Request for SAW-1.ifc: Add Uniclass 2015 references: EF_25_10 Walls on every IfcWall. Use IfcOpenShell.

First a look at what the model holds.

```python
import ifcopenshell

model = ifcopenshell.open("SAW-1.ifc")
print(model.schema)
print("classifications:", [c.Name for c in model.by_type("IfcClassification")])
for ifc_class in ("IfcDoor", "IfcRoof", "IfcStair", "IfcWall", "IfcWindow"):
    print(ifc_class, len(model.by_type(ifc_class)))
```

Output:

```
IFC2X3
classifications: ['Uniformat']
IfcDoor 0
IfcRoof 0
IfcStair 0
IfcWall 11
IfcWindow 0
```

```python
import ifcopenshell
import ifcopenshell.api.classification

model = ifcopenshell.open("SAW-1.ifc")

# IFC2X3 requires Source and Edition and has no link from the project to the system.
system = model.create_entity("IfcClassification", Source="NBS", Edition="2015", Name="Uniclass 2015")

codes = {
    "IfcWall": ("EF_25_10", "Walls"),
}
for ifc_class, (code, name) in codes.items():
    products = model.by_type(ifc_class)
    ifcopenshell.api.classification.add_reference(
        model, products=products, classification=system, identification=code, name=name
    )
    print(code, len(products))

model.write("SAW-1-out.ifc")
```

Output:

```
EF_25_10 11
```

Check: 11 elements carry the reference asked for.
